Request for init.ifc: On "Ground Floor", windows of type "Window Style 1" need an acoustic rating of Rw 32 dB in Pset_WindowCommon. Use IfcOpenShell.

First a look at what the model holds.

```python
import ifcopenshell
import ifcopenshell.util.element

model = ifcopenshell.open("init.ifc")
print(model.schema)
storey = next(s for s in model.by_type("IfcBuildingStorey") if s.Name == "Ground Floor")
windows = [e for e in ifcopenshell.util.element.get_decomposition(storey) if e.is_a("IfcWindow")]
seen = {}
for e in windows:
    element_type = ifcopenshell.util.element.get_type(e)
    key = (element_type.Name if element_type != e and element_type else None, ifcopenshell.util.element.get_pset(e, "Pset_WindowCommon", "AcousticRating"))
    seen[key] = seen.get(key, 0) + 1
for (name, value), count in sorted(seen.items(), key=str):
    print(count, "x", name, "|", value)
```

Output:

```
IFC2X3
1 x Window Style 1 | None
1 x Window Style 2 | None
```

```python
import ifcopenshell
import ifcopenshell.api.pset
import ifcopenshell.util.element

model = ifcopenshell.open("init.ifc")

storey = next(s for s in model.by_type("IfcBuildingStorey") if s.Name == "Ground Floor")
windows = [e for e in ifcopenshell.util.element.get_decomposition(storey) if e.is_a("IfcWindow")]

count = 0
for e in windows:
    element_type = ifcopenshell.util.element.get_type(e)
    if element_type in (None, e) or element_type.Name != "Window Style 1":
        continue
    # add_pset returns the element's existing set when there is one.
    pset = ifcopenshell.api.pset.add_pset(model, product=e, name="Pset_WindowCommon")
    ifcopenshell.api.pset.edit_pset(model, pset=pset, properties={"AcousticRating": "Rw 32 dB"})
    count += 1

print(count, "windows updated")

model.write("init_v2.ifc")
```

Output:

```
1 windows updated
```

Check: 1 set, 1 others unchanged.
